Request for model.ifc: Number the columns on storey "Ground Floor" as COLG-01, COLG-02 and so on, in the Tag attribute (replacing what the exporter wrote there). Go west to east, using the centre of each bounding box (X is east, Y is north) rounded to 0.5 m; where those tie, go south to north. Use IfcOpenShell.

First a look at what the model holds.

```python
import ifcopenshell
import ifcopenshell.util.element
import ifcopenshell.util.placement

model = ifcopenshell.open("model.ifc")
print(model.schema)
storey = next(s for s in model.by_type("IfcBuildingStorey") if s.Name == "Ground Floor")
columns = [e for e in ifcopenshell.util.element.get_decomposition(storey) if e.is_a("IfcColumn")]
for e in sorted(columns, key=lambda e: e.id()):
    origin = ifcopenshell.util.placement.get_local_placement(e.ObjectPlacement)[:3, 3]
    print(e.id(), e.Tag, e.Name, origin.round(2) + 0.0, sep=" | ")
```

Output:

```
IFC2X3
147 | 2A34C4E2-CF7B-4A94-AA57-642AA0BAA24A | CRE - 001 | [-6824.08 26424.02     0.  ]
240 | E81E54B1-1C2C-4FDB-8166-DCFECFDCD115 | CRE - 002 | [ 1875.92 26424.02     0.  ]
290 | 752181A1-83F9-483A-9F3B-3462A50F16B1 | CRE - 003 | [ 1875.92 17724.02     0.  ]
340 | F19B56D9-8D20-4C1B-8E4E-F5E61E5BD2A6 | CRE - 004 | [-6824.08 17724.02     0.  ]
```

```python
import ifcopenshell
import ifcopenshell.geom
import ifcopenshell.util.element
import ifcopenshell.util.shape

model = ifcopenshell.open("model.ifc")
settings = ifcopenshell.geom.settings()
settings.set("use-world-coords", True)


def centre(element):
    shape = ifcopenshell.geom.create_shape(settings, element)
    return ifcopenshell.util.shape.get_bbox_centroid(shape.geometry)


storey = next(s for s in model.by_type("IfcBuildingStorey") if s.Name == "Ground Floor")
columns = [e for e in ifcopenshell.util.element.get_decomposition(storey) if e.is_a("IfcColumn")]

# Insertion points can sit at a corner or the storey origin, so sort by the geometry (in metres).
centres = {e: centre(e) for e in columns}
columns.sort(key=lambda e: (round(centres[e][0] / 0.5), centres[e][1]))

for i, e in enumerate(columns, start=1):
    number = f"COLG-{i:02d}"
    e.Tag = number
    print(e.id(), number)

model.write("model-out.ifc")
```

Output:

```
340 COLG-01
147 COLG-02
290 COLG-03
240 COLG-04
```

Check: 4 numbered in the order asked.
